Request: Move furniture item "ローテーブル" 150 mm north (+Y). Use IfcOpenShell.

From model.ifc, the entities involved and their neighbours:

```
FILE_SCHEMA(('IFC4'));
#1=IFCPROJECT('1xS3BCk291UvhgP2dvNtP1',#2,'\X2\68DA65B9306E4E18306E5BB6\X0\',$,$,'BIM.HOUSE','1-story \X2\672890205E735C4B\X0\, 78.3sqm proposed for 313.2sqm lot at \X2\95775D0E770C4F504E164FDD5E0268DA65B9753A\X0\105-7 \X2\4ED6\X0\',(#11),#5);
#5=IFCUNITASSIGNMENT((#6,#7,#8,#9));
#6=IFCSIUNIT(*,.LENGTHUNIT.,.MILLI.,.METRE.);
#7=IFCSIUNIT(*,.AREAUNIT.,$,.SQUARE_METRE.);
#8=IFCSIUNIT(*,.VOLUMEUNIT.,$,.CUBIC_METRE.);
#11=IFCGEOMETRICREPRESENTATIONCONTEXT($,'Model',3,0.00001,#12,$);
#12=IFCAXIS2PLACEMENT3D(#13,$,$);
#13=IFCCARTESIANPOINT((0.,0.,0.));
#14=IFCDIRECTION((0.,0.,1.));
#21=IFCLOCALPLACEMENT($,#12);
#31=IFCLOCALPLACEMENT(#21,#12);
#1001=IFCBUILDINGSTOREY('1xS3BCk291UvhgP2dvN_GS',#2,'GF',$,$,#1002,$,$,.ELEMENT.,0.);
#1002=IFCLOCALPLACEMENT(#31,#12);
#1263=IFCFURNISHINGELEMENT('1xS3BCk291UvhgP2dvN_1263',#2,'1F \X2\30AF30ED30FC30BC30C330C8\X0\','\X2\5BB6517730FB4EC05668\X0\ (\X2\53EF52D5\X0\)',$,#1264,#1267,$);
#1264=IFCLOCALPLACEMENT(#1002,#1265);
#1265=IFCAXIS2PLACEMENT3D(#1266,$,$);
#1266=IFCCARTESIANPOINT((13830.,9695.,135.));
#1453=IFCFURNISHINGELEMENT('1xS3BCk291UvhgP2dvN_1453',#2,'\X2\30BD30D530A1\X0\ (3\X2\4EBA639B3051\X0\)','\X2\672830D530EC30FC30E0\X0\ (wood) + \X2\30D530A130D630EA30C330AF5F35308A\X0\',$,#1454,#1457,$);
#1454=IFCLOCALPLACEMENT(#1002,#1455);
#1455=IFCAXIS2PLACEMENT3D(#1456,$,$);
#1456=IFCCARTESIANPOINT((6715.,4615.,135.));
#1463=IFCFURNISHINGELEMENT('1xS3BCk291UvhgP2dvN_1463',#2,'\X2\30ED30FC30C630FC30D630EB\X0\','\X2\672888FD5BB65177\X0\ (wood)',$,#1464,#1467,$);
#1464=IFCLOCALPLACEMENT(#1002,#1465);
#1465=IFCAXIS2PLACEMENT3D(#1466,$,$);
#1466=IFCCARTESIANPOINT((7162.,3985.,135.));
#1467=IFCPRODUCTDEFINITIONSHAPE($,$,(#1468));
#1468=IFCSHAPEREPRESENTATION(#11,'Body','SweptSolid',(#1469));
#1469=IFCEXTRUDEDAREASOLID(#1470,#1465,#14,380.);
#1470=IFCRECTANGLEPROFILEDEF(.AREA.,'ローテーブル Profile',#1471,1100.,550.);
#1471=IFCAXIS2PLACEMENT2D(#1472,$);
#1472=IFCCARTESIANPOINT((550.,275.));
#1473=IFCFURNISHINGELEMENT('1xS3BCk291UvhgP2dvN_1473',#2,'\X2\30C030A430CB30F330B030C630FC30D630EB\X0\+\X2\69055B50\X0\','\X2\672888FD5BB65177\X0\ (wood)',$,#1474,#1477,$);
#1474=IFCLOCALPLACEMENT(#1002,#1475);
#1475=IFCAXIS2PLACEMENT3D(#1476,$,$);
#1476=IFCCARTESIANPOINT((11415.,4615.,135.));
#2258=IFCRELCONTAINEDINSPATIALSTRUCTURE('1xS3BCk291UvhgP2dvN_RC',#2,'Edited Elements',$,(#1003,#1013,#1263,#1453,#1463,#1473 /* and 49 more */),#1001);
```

```python
import ifcopenshell
import ifcopenshell.api.geometry
import ifcopenshell.util.placement

model = ifcopenshell.open("model.ifc")

item = model.by_id(1463)
matrix = ifcopenshell.util.placement.get_local_placement(item.ObjectPlacement)
matrix[1, 3] += 150.0
ifcopenshell.api.geometry.edit_object_placement(model, product=item, matrix=matrix, is_si=False)

print(ifcopenshell.util.placement.get_local_placement(item.ObjectPlacement).round(3) + 0.0)

model.write("model_updated.ifc")
```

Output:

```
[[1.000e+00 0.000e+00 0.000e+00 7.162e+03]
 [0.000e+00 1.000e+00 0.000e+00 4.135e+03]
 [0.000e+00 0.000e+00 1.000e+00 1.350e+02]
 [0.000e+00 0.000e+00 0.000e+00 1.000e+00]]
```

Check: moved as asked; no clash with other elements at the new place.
